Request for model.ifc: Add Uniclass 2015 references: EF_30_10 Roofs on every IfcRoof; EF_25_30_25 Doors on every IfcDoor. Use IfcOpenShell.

First a look at what the model holds.

```python
import ifcopenshell

model = ifcopenshell.open("model.ifc")
print(model.schema)
print("classifications:", [c.Name for c in model.by_type("IfcClassification")])
for ifc_class in ("IfcDoor", "IfcRoof", "IfcStair", "IfcWall", "IfcWindow"):
    print(ifc_class, len(model.by_type(ifc_class)))
```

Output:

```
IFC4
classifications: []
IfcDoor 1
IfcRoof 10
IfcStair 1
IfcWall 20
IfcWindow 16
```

```python
import ifcopenshell
import ifcopenshell.api.classification

model = ifcopenshell.open("model.ifc")

system = ifcopenshell.api.classification.add_classification(model, classification="Uniclass 2015")

codes = {
    "IfcRoof": ("EF_30_10", "Roofs"),
    "IfcDoor": ("EF_25_30_25", "Doors"),
}
for ifc_class, (code, name) in codes.items():
    products = model.by_type(ifc_class)
    ifcopenshell.api.classification.add_reference(
        model, products=products, classification=system, identification=code, name=name
    )
    print(code, len(products))

model.write("model_edited.ifc")
```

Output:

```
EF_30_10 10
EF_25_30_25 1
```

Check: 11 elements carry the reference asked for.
